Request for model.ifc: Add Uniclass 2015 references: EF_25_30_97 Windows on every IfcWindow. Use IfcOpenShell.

First a look at what the model holds.

```python
import ifcopenshell

model = ifcopenshell.open("model.ifc")
print(model.schema)
print("classifications:", [c.Name for c in model.by_type("IfcClassification")])
for ifc_class in ("IfcDoor", "IfcRoof", "IfcStair", "IfcWall", "IfcWindow"):
    print(ifc_class, len(model.by_type(ifc_class)))
```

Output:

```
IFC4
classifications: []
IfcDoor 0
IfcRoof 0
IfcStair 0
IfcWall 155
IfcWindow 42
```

```python
import ifcopenshell
import ifcopenshell.api.classification

model = ifcopenshell.open("model.ifc")

system = ifcopenshell.api.classification.add_classification(model, classification="Uniclass 2015")

codes = {
    "IfcWindow": ("EF_25_30_97", "Windows"),
}
for ifc_class, (code, name) in codes.items():
    products = model.by_type(ifc_class)
    ifcopenshell.api.classification.add_reference(
        model, products=products, classification=system, identification=code, name=name
    )
    print(code, len(products))

model.write("model_updated.ifc")
```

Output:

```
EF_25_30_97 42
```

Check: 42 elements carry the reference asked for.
